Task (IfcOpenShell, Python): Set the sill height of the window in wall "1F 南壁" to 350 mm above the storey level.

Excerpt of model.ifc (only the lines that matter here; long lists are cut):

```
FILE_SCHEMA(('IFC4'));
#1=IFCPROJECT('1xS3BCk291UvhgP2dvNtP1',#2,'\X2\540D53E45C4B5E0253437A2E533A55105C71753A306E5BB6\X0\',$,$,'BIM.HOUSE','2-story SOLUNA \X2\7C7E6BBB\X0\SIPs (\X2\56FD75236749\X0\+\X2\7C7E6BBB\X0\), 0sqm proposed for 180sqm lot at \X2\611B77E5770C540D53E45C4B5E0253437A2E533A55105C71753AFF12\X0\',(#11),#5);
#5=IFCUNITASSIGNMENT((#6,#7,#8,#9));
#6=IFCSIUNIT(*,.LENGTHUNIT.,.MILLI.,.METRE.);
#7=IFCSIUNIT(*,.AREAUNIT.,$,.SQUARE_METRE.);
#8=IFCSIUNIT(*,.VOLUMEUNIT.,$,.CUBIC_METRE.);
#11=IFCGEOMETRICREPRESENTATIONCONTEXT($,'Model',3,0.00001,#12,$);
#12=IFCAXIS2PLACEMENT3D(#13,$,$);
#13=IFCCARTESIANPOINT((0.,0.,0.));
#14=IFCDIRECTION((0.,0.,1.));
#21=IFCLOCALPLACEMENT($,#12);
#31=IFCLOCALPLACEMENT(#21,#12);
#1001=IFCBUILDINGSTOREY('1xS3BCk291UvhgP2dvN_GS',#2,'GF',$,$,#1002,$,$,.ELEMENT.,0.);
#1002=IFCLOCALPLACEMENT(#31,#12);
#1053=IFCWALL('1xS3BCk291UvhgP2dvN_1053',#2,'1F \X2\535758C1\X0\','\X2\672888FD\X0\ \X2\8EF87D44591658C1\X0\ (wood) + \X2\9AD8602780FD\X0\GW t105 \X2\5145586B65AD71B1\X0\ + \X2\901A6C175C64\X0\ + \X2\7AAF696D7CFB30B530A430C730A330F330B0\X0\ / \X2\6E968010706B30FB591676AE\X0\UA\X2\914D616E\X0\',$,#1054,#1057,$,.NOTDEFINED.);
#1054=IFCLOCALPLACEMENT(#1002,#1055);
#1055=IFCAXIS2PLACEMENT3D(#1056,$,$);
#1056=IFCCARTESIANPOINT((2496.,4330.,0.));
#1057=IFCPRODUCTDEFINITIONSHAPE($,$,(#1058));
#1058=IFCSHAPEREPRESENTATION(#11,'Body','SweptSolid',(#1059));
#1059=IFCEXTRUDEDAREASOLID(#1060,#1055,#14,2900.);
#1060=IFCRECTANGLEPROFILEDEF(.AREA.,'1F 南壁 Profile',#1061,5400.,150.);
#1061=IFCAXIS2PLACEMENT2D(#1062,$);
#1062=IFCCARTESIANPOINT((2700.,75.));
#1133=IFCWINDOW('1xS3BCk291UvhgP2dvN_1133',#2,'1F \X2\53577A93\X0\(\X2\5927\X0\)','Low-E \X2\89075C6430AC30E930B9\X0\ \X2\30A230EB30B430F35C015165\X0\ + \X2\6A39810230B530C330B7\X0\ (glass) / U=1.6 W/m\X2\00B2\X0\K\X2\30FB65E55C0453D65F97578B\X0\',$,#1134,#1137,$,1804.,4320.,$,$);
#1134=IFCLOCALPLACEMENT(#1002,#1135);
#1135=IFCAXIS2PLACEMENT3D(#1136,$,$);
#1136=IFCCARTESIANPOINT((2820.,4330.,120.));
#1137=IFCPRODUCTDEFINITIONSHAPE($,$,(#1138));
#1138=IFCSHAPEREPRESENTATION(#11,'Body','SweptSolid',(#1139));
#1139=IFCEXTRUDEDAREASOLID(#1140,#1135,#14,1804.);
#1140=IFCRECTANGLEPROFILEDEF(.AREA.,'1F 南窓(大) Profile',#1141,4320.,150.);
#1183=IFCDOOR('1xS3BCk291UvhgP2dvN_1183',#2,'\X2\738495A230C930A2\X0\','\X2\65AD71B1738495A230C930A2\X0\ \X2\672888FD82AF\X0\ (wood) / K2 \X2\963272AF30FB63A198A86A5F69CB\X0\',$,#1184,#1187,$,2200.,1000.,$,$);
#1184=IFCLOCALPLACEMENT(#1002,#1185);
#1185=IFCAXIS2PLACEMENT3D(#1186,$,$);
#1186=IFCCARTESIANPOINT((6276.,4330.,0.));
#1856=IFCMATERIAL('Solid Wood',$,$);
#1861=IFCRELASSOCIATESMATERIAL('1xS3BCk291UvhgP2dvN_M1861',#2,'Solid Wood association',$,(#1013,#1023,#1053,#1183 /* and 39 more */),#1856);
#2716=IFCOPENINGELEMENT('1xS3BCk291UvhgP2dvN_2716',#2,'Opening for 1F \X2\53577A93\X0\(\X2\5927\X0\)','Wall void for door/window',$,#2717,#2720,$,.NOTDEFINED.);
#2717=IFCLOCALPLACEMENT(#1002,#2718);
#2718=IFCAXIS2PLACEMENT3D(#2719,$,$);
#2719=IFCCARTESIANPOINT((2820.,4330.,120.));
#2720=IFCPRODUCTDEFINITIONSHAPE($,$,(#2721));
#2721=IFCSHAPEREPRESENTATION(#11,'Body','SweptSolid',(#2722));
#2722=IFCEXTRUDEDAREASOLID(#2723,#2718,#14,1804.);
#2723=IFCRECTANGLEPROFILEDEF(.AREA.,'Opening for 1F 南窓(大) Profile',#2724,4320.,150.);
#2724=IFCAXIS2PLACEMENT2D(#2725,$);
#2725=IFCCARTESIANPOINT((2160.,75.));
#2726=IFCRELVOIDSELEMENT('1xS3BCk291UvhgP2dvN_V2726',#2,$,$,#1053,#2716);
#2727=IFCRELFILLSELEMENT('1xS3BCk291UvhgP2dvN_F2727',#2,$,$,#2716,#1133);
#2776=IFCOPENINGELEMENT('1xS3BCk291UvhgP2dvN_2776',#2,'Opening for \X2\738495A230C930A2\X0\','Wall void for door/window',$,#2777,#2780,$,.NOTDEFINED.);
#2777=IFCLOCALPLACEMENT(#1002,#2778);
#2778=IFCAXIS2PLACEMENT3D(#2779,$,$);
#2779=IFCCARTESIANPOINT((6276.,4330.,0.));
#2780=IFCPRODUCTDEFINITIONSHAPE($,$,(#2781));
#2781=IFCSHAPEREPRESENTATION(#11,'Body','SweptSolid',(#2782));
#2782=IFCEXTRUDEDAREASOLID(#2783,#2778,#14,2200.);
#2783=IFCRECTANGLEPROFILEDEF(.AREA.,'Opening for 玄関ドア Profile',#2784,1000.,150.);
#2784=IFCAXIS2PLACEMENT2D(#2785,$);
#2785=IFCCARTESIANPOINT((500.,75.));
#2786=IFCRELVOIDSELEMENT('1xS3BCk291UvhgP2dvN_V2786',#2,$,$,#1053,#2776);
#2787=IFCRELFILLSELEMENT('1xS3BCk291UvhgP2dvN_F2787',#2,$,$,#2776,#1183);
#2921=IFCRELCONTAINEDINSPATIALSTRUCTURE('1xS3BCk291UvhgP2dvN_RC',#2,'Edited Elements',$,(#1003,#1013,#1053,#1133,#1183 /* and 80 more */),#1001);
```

```python
import numpy as np
import ifcopenshell
import ifcopenshell.api.geometry
import ifcopenshell.geom
import ifcopenshell.util.element
import ifcopenshell.util.placement
import ifcopenshell.util.shape
import ifcopenshell.util.unit

model = ifcopenshell.open("model.ifc")
unit_scale = ifcopenshell.util.unit.calculate_unit_scale(model)

window = model.by_guid("1xS3BCk291UvhgP2dvN_1133")
opening = window.FillsVoids[0].RelatingOpeningElement
storey = ifcopenshell.util.element.get_container(window, ifc_class="IfcBuildingStorey")
level = ifcopenshell.util.placement.get_local_placement(storey.ObjectPlacement)[2, 3]

# The opening's origin need not be at the sill, so measure its lowest point.
shape = ifcopenshell.geom.create_shape(ifcopenshell.geom.settings(), opening)
bottom = ifcopenshell.util.shape.get_shape_bottom_elevation(shape, shape.geometry) / unit_scale
dz = level + 350.0 - bottom

shift = np.array([0.0, 0.0, dz])
# The window is not placed relative to its opening, so move both.
for product in (opening, window):
    matrix = ifcopenshell.util.placement.get_local_placement(product.ObjectPlacement)
    matrix[:3, 3] += shift
    ifcopenshell.api.geometry.edit_object_placement(model, product=product, matrix=matrix, is_si=False)

print(f"moved by {dz * unit_scale:+.3f} m")

model.write("model_updated.ifc")
```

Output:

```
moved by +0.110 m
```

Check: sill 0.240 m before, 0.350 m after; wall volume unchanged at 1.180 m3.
